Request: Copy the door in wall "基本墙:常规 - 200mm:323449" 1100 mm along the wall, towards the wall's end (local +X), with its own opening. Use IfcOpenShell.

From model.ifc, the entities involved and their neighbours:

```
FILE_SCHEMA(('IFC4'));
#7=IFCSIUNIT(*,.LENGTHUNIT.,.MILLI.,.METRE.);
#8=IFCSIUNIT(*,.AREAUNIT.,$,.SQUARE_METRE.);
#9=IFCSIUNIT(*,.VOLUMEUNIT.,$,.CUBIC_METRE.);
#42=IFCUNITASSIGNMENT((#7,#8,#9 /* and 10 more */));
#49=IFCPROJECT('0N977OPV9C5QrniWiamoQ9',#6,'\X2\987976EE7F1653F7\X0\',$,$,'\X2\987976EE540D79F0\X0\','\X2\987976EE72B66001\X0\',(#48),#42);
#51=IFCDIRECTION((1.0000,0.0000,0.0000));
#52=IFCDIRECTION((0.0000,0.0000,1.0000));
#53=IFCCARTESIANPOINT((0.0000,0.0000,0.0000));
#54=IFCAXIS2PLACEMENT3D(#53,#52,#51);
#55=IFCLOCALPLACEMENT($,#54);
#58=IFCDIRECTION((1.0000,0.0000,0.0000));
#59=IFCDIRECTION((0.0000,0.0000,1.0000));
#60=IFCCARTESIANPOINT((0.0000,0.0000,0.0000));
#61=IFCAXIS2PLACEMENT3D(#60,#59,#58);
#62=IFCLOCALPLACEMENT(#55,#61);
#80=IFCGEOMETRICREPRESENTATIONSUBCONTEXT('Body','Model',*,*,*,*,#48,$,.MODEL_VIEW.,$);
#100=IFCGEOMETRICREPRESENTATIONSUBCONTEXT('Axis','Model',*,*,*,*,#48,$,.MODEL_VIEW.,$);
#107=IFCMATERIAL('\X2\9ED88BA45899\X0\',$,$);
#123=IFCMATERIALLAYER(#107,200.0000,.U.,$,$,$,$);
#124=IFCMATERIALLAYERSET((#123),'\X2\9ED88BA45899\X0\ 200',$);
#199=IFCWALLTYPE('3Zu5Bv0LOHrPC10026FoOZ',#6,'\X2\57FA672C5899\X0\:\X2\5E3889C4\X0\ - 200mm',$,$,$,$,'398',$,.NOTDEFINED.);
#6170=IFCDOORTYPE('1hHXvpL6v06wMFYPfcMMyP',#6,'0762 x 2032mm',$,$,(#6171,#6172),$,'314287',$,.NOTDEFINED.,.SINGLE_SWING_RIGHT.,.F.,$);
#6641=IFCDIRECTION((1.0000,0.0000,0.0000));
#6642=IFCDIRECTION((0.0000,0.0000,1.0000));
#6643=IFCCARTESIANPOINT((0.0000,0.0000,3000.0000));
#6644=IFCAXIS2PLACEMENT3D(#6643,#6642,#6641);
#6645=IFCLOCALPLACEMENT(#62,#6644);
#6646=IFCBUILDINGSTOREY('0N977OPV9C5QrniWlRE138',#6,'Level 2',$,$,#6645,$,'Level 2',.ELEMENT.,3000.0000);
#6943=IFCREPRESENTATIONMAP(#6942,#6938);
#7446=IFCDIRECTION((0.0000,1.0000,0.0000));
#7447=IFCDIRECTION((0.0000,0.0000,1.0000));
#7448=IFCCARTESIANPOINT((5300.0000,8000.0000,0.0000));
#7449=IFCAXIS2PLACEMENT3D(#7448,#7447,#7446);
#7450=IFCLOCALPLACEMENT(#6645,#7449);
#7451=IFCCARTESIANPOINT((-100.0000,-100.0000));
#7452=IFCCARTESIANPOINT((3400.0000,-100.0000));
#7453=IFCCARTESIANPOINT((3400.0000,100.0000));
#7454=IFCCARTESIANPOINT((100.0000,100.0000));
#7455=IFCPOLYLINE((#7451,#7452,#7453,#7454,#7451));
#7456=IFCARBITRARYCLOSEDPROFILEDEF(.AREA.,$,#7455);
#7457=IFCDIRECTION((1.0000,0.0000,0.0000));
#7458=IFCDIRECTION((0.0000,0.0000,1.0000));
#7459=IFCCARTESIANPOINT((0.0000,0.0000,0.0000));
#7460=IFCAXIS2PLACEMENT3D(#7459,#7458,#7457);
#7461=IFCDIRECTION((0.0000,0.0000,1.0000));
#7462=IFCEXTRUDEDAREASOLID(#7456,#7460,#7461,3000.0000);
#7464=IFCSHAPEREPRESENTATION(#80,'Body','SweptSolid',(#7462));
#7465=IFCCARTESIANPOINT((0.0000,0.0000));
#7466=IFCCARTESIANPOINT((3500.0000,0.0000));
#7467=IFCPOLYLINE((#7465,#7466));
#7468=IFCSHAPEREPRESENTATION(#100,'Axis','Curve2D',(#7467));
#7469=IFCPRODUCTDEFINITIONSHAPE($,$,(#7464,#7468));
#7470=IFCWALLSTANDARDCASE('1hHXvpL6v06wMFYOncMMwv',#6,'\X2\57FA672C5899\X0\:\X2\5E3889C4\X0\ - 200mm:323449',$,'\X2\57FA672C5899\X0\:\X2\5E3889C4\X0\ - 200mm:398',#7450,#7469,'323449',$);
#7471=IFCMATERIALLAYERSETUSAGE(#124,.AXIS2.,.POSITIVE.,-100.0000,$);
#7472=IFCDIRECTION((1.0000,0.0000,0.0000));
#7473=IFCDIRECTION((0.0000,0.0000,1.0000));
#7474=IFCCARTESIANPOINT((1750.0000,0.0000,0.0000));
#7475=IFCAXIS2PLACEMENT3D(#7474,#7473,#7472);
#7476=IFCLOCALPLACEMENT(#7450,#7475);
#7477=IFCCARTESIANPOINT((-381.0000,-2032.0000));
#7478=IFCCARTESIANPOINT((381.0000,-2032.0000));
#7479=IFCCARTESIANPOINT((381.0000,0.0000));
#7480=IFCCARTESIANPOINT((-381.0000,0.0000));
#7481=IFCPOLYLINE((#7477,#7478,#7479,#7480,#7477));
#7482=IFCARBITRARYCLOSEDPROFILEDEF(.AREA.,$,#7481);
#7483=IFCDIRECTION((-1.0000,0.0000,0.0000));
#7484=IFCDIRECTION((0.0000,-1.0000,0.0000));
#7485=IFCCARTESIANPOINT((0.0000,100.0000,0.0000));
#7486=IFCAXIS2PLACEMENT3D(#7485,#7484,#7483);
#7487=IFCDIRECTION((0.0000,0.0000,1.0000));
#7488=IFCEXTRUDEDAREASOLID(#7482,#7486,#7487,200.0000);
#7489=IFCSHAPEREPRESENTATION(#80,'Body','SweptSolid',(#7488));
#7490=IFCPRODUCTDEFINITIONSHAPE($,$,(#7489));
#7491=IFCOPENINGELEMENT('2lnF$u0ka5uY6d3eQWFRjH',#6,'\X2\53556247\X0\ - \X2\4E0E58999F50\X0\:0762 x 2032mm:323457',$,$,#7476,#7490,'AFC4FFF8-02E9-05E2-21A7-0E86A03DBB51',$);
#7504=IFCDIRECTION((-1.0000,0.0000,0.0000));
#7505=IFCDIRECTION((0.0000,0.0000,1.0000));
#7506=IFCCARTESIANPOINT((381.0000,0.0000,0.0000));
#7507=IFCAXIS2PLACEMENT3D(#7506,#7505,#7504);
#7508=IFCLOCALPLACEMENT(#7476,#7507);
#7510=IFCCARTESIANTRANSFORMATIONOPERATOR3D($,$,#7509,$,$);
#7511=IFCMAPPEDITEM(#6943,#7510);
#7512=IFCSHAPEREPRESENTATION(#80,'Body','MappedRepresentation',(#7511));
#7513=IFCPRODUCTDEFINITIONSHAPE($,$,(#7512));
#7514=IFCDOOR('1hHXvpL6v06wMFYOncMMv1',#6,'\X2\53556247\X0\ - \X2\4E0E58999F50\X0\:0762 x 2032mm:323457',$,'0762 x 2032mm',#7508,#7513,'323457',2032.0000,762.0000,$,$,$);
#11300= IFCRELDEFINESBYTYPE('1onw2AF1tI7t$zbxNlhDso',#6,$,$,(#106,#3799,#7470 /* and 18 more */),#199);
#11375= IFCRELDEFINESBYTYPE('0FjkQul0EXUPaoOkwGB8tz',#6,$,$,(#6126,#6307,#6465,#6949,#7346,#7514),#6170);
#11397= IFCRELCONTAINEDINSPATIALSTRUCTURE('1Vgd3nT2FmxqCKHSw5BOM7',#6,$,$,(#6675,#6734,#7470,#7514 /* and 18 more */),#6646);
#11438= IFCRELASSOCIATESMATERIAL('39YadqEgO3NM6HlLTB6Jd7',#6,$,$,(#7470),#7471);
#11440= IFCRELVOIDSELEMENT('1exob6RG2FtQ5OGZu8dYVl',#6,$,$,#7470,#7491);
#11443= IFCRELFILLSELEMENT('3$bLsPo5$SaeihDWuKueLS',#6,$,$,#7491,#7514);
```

```python
import ifcopenshell
import ifcopenshell.api.feature
import ifcopenshell.api.geometry
import ifcopenshell.api.root
import ifcopenshell.geom
import ifcopenshell.util.element
import ifcopenshell.util.placement
import ifcopenshell.util.shape
import ifcopenshell.util.unit

model = ifcopenshell.open("model.ifc")
unit_scale = ifcopenshell.util.unit.calculate_unit_scale(model)
settings = ifcopenshell.geom.settings()


def volume(element):
    """Net volume in cubic metres, openings subtracted."""
    shape = ifcopenshell.geom.create_shape(settings, element)
    return ifcopenshell.util.shape.get_volume(shape.geometry)


def reuse_history(source, copy):
    """copy_class also copies each property set's owner history, people and application; keep the originals."""
    for rel in copy.IsDefinedBy:
        if rel.is_a("IfcRelDefinesByProperties") and (history := rel.RelatingPropertyDefinition.OwnerHistory):
            rel.RelatingPropertyDefinition.OwnerHistory = source.OwnerHistory
            ifcopenshell.util.element.remove_deep2(model, history)


door = model.by_id(7514)
opening = door.FillsVoids[0].RelatingOpeningElement
wall = opening.VoidsElements[0].RelatingBuildingElement
before = volume(wall)
shift = ifcopenshell.util.placement.get_local_placement(wall.ObjectPlacement)[:3, 0] * 1.1 / unit_scale

# copy_class copies the void relationship, type, container and properties, but no geometry.
new_opening = ifcopenshell.api.root.copy_class(model, product=opening)
new_opening.Representation = ifcopenshell.util.element.copy_deep(
    model, opening.Representation, exclude=["IfcGeometricRepresentationContext", "IfcRepresentationMap"]
)
new_opening.Name = "单扇 - 与墙齐:0762 x 2032mm"
new_opening.Tag = None
new_door = ifcopenshell.api.root.copy_class(model, product=door)
new_door.Representation = ifcopenshell.util.element.copy_deep(
    model, door.Representation, exclude=["IfcGeometricRepresentationContext", "IfcRepresentationMap"]
)
new_door.Name = "单扇 - 与墙齐:0762 x 2032mm"
new_door.Tag = None
reuse_history(door, new_door)
ifcopenshell.api.feature.add_filling(model, opening=new_opening, element=new_door)

for old, new in ((opening, new_opening), (door, new_door)):
    matrix = ifcopenshell.util.placement.get_local_placement(old.ObjectPlacement)
    matrix[:3, 3] += shift
    ifcopenshell.api.geometry.edit_object_placement(model, product=new, matrix=matrix, is_si=False)

after = volume(wall)

print(f"wall volume {before:.3f} -> {after:.3f} m3")

model.write("model-out.ifc")
```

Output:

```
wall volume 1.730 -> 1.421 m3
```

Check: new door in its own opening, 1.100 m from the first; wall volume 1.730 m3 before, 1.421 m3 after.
